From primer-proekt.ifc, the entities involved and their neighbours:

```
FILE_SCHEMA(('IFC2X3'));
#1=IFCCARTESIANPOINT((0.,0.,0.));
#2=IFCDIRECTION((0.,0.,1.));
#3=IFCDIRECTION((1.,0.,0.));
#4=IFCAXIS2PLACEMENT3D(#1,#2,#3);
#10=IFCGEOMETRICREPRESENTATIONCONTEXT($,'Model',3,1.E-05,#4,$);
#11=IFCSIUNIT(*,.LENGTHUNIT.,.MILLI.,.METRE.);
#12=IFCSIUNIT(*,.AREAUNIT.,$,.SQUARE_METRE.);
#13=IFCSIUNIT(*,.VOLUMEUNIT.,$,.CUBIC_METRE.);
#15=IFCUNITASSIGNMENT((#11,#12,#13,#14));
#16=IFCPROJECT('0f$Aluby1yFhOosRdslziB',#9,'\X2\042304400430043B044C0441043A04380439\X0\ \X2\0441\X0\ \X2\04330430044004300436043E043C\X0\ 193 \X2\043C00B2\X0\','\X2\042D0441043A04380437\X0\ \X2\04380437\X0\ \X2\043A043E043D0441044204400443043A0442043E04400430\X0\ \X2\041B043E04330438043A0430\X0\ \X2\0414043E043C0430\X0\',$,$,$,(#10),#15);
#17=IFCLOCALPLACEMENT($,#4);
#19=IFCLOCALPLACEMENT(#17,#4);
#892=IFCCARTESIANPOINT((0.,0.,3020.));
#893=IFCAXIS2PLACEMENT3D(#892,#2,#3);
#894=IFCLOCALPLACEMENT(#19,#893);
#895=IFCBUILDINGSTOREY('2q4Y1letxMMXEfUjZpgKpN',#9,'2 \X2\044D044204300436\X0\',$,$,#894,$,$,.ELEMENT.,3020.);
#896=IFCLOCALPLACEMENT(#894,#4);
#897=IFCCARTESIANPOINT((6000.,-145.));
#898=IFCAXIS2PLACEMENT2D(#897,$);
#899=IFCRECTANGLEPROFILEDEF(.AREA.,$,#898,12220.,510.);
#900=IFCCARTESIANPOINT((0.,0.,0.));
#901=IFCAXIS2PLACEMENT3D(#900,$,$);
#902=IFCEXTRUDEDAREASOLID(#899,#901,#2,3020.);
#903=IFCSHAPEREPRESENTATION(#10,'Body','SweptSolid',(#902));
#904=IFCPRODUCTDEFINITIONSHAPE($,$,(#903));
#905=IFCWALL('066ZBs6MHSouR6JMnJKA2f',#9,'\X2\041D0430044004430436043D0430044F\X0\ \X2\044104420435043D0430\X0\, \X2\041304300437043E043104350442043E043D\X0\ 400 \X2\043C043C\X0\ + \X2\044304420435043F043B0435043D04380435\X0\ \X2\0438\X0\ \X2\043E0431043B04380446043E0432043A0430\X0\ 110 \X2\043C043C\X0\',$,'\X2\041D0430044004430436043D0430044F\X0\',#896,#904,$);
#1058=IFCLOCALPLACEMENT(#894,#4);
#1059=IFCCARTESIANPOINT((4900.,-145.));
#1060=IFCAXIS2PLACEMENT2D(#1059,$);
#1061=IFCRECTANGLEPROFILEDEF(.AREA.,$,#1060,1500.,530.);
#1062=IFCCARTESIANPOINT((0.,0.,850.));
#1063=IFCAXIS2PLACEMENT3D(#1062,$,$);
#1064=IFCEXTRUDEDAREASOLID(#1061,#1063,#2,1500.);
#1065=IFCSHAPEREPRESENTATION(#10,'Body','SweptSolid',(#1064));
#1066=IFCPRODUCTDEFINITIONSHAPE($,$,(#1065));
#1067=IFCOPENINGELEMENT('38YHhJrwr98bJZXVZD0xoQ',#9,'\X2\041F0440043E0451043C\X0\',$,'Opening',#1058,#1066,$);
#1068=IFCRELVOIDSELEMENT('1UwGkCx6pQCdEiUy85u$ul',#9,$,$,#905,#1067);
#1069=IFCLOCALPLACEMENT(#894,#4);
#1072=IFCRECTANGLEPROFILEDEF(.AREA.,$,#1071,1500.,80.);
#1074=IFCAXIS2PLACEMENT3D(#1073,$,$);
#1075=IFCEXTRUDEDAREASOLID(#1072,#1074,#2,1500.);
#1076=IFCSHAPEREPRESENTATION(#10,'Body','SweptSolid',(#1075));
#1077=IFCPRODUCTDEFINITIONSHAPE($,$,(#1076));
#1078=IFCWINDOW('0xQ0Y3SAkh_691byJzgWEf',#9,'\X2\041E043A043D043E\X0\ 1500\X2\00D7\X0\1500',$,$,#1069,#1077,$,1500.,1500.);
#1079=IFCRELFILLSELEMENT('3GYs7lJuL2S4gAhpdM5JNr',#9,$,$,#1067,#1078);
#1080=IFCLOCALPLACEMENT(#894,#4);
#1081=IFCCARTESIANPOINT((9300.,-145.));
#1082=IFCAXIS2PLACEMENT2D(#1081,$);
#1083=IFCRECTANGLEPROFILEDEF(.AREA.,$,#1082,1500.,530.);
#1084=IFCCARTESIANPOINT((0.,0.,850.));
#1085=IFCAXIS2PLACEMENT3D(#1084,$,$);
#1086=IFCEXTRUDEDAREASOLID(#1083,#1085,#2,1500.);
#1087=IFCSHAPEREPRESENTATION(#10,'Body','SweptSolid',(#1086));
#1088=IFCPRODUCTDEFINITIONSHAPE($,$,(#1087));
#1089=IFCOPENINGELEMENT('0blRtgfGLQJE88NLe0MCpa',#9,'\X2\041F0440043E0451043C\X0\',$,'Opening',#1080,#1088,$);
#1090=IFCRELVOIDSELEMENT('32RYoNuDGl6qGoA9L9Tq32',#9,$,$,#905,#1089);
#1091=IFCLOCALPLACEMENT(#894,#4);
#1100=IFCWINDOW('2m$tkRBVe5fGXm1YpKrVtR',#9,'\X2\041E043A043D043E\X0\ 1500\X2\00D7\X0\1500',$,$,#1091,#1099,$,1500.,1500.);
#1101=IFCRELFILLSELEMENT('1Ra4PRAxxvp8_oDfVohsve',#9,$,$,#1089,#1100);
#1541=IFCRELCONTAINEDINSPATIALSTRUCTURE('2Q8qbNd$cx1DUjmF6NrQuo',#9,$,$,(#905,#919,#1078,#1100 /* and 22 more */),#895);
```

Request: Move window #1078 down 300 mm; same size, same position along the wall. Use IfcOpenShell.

```python
import numpy as np
import ifcopenshell
import ifcopenshell.api.geometry
import ifcopenshell.util.placement
import ifcopenshell.util.unit

model = ifcopenshell.open("primer-proekt.ifc")
unit_scale = ifcopenshell.util.unit.calculate_unit_scale(model)

window = model.by_id(1078)
opening = window.FillsVoids[0].RelatingOpeningElement
dz = -0.3 / unit_scale

shift = np.array([0.0, 0.0, dz])
# The window is not placed relative to its opening, so move both.
for product in (opening, window):
    matrix = ifcopenshell.util.placement.get_local_placement(product.ObjectPlacement)
    matrix[:3, 3] += shift
    ifcopenshell.api.geometry.edit_object_placement(model, product=product, matrix=matrix, is_si=False)

print(f"moved by {dz * unit_scale:+.3f} m")

model.write("primer-proekt_updated.ifc")
```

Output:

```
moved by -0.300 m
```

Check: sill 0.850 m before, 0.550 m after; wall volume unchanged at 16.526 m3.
